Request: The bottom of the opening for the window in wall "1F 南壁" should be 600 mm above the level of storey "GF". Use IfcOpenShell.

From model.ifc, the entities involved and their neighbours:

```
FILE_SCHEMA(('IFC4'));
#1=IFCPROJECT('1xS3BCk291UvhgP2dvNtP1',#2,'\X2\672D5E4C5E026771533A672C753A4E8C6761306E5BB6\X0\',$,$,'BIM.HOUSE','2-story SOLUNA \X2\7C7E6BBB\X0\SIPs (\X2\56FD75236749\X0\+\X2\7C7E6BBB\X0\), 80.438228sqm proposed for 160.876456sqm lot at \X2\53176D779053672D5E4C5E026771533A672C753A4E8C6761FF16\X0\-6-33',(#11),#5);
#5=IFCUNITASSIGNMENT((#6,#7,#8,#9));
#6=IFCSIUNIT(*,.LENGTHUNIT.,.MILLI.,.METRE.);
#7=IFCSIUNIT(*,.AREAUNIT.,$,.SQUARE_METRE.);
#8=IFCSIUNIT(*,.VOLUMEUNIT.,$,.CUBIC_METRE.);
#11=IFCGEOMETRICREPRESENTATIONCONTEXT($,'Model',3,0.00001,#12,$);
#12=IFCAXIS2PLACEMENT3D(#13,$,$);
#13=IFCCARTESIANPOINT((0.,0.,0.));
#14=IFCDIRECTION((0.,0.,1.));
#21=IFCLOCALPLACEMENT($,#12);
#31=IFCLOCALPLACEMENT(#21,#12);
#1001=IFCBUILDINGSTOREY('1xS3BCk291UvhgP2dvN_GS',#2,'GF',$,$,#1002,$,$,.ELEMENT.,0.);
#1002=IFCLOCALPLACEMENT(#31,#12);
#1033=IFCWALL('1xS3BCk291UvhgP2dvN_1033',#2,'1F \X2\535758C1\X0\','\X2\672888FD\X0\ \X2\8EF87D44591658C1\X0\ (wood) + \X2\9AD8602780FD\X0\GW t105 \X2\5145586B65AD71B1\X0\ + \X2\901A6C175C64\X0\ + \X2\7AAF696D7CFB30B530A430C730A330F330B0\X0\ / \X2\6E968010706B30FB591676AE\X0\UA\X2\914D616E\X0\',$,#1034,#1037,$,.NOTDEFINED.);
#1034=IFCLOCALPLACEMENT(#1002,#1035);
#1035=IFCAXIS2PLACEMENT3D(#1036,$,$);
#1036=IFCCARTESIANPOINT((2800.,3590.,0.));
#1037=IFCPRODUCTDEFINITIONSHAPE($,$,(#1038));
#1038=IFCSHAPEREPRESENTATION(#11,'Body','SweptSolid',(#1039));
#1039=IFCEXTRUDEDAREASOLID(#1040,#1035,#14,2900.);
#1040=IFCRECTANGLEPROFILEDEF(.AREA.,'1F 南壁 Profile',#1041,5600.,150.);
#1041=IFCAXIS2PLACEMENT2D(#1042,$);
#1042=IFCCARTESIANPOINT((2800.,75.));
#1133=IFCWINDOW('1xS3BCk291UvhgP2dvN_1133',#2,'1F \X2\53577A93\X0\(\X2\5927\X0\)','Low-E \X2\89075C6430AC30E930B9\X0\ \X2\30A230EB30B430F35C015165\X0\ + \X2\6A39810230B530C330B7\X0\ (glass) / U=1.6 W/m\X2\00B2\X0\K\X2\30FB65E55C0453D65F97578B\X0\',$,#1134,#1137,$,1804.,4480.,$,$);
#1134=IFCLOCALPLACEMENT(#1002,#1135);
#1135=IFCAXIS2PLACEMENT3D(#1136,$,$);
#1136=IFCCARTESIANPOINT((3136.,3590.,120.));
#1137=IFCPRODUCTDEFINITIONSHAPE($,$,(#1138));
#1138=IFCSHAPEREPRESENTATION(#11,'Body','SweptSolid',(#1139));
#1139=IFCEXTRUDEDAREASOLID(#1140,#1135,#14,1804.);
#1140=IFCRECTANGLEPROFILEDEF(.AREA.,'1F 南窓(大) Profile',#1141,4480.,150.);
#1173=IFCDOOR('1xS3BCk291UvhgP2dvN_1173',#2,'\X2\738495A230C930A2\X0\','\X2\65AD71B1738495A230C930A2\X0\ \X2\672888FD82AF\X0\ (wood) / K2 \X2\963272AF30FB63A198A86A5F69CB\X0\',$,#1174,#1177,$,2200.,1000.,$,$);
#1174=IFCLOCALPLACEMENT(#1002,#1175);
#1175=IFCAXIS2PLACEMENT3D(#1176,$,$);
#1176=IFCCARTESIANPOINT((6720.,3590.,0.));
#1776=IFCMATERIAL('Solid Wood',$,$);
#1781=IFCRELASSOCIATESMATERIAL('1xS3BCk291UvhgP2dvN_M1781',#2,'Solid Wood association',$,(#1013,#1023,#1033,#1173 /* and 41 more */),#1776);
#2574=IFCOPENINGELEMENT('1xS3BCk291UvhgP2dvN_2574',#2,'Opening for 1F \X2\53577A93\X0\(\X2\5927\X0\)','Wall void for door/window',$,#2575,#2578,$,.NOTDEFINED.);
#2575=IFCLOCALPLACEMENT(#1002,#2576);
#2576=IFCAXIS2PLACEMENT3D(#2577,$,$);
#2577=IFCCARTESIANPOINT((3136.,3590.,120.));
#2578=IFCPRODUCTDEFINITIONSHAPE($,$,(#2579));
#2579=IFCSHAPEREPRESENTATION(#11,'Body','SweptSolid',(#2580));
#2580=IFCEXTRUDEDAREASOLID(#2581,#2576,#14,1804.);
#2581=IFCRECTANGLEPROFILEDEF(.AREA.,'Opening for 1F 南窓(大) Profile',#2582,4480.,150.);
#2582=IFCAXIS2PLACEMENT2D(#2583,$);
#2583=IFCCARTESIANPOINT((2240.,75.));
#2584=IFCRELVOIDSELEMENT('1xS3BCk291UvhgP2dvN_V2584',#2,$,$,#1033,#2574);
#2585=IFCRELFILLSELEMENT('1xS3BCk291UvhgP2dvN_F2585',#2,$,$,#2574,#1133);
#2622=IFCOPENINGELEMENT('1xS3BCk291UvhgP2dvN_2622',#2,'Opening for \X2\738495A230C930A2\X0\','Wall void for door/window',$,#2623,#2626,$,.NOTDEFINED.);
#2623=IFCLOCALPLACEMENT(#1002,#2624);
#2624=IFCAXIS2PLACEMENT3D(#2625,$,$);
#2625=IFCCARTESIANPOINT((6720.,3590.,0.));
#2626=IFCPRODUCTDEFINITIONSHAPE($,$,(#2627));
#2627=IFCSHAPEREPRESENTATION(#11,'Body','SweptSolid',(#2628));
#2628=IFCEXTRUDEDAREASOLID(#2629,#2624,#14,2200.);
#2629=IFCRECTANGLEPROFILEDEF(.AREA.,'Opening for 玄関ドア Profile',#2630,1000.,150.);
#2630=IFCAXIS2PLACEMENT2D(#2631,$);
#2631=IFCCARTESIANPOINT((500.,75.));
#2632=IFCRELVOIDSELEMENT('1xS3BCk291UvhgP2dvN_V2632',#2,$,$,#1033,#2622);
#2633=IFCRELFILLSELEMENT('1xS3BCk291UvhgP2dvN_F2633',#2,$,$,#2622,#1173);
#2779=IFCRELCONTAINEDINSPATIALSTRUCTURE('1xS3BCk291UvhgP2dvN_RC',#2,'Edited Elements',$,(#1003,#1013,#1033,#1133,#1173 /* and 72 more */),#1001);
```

```python
import numpy as np
import ifcopenshell
import ifcopenshell.api.geometry
import ifcopenshell.geom
import ifcopenshell.util.element
import ifcopenshell.util.placement
import ifcopenshell.util.shape
import ifcopenshell.util.unit

model = ifcopenshell.open("model.ifc")
unit_scale = ifcopenshell.util.unit.calculate_unit_scale(model)

window = model.by_id(1133)
opening = window.FillsVoids[0].RelatingOpeningElement
storey = ifcopenshell.util.element.get_container(window, ifc_class="IfcBuildingStorey")
level = ifcopenshell.util.placement.get_local_placement(storey.ObjectPlacement)[2, 3]

# The opening's origin need not be at the sill, so measure its lowest point.
shape = ifcopenshell.geom.create_shape(ifcopenshell.geom.settings(), opening)
bottom = ifcopenshell.util.shape.get_shape_bottom_elevation(shape, shape.geometry) / unit_scale
dz = level + 600.0 - bottom

shift = np.array([0.0, 0.0, dz])
# The window is not placed relative to its opening, so move both.
for product in (opening, window):
    matrix = ifcopenshell.util.placement.get_local_placement(product.ObjectPlacement)
    matrix[:3, 3] += shift
    ifcopenshell.api.geometry.edit_object_placement(model, product=product, matrix=matrix, is_si=False)

print(f"moved by {dz * unit_scale:+.3f} m")

model.write("model_edited.ifc")
```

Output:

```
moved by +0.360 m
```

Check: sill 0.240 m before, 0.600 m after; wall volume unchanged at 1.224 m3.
